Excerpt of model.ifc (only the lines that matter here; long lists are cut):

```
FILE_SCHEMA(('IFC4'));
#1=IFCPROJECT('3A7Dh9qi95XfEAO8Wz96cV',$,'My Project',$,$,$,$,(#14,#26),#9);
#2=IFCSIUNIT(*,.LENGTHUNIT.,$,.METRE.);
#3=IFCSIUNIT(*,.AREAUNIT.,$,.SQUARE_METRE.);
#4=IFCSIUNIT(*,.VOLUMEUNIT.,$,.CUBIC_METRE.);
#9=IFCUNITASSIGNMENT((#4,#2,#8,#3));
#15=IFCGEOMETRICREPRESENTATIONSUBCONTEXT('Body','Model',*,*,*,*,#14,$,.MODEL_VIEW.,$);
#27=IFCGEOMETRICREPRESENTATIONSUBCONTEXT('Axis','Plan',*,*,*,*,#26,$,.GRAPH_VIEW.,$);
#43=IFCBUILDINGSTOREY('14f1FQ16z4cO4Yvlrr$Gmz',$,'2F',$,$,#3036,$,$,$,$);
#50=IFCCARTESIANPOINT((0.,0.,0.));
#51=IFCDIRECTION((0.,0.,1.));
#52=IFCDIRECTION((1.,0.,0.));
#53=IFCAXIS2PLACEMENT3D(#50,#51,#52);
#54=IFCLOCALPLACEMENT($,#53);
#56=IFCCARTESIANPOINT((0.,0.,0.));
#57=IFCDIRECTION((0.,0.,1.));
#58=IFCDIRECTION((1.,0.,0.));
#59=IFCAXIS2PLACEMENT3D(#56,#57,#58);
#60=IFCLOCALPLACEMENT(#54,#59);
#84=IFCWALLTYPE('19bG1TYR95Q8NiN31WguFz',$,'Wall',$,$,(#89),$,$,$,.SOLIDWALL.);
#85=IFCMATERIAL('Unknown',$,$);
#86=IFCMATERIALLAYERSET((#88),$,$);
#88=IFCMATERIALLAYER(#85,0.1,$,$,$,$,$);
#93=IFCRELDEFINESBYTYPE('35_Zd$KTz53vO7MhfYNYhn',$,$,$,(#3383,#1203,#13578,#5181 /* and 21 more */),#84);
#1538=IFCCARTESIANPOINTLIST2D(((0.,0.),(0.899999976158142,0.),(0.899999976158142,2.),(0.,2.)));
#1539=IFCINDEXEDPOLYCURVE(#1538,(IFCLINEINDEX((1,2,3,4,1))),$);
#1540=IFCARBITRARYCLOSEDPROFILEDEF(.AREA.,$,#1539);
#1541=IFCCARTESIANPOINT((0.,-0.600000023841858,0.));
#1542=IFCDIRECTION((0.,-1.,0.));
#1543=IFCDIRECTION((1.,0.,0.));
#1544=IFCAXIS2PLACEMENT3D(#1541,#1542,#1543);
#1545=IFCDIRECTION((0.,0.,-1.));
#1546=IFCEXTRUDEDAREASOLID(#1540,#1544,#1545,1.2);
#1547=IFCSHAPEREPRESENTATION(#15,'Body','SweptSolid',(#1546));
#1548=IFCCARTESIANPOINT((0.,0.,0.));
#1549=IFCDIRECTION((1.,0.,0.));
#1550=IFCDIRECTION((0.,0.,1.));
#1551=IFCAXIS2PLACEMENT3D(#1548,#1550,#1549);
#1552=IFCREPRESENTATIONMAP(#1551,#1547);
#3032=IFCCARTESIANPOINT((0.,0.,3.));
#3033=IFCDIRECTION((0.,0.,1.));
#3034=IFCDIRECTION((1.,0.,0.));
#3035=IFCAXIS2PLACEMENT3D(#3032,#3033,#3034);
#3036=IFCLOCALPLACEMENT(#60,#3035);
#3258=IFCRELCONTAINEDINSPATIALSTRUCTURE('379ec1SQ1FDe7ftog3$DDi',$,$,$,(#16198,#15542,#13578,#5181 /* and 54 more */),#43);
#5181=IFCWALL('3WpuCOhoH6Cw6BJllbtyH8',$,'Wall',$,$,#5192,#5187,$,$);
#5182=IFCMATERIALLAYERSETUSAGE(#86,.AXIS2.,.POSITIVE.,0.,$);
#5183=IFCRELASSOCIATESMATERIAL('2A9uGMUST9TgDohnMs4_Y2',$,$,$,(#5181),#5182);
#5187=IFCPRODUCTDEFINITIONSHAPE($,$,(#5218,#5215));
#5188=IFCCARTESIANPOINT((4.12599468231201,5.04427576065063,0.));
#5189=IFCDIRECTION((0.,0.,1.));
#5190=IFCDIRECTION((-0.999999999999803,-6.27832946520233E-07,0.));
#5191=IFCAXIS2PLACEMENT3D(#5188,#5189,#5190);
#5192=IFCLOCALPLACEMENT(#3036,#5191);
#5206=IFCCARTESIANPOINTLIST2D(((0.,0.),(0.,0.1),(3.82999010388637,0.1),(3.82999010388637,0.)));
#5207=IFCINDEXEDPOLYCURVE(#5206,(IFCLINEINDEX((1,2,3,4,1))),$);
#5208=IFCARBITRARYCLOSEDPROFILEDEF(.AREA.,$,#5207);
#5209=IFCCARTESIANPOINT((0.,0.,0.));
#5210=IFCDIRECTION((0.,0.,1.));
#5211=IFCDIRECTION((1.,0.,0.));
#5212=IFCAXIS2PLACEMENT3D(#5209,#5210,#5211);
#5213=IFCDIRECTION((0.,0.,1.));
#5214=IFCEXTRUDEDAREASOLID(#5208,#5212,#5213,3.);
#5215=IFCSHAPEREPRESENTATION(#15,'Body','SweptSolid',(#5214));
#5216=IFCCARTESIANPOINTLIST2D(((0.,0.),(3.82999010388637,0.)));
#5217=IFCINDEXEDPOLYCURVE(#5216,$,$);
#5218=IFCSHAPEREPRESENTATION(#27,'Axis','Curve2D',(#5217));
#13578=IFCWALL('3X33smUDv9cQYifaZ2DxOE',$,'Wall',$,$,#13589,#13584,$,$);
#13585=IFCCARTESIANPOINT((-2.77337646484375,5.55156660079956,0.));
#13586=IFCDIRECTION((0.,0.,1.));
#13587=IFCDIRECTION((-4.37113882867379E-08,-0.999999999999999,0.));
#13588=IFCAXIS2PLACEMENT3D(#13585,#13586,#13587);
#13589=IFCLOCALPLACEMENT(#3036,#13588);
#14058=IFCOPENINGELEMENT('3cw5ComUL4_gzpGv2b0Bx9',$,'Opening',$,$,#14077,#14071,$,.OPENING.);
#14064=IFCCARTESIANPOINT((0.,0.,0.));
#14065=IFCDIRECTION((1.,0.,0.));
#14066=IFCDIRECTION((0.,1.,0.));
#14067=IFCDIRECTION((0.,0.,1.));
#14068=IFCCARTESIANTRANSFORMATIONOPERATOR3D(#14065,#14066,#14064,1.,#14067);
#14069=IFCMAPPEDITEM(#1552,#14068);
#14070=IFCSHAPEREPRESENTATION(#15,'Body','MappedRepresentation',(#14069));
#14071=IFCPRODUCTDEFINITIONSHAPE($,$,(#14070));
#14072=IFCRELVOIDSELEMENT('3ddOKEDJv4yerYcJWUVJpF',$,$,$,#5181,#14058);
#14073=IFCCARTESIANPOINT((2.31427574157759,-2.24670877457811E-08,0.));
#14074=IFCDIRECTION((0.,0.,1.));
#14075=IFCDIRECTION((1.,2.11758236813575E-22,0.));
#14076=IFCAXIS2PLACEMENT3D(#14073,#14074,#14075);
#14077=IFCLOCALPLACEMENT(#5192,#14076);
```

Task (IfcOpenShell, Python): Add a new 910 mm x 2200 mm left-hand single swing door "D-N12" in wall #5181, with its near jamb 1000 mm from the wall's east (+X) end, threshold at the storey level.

```python
import numpy as np
import ifcopenshell
import ifcopenshell.api.feature
import ifcopenshell.api.geometry
import ifcopenshell.api.root
import ifcopenshell.api.spatial
import ifcopenshell.geom
import ifcopenshell.util.element
import ifcopenshell.util.placement
import ifcopenshell.util.representation
import ifcopenshell.util.shape
import ifcopenshell.util.unit

model = ifcopenshell.open("model.ifc")
unit_scale = ifcopenshell.util.unit.calculate_unit_scale(model)
settings = ifcopenshell.geom.settings()


def volume(element):
    """Net volume in cubic metres, openings subtracted."""
    shape = ifcopenshell.geom.create_shape(settings, element)
    return ifcopenshell.util.shape.get_volume(shape.geometry)


wall = model.by_guid("3WpuCOhoH6Cw6BJllbtyH8")
storey = ifcopenshell.util.element.get_container(wall, ifc_class="IfcBuildingStorey")
context = ifcopenshell.util.representation.get_context(model, "Model", "Body", "MODEL_VIEW")
before = volume(wall)

width, height, from_end, sill = 0.91, 2.2, 1, 0.0  # metres

# The wall runs along its own X axis, and the end named is its -X end.
wall_shape = ifcopenshell.geom.create_shape(settings, wall)
x, y, z = ifcopenshell.util.shape.get_vertices(wall_shape.geometry).T
start = x.min() + from_end
face, thickness = float(y.min()), float(y.max() - y.min())
wall_matrix = ifcopenshell.util.placement.get_local_placement(wall.ObjectPlacement)
level = ifcopenshell.util.placement.get_local_placement(storey.ObjectPlacement)[2, 3]


def in_wall(x, y):
    """Placement at x, y metres in the wall's axes, at sill height."""
    matrix = wall_matrix.copy()
    matrix[:, 3] = wall_matrix @ np.array([x / unit_scale, y / unit_scale, 0.0, 1.0])
    matrix[2, 3] = level + sill / unit_scale
    return matrix


# Opening: a box that overshoots both wall faces by 50 mm.
opening = ifcopenshell.api.root.create_entity(model, ifc_class="IfcOpeningElement", predefined_type="OPENING")
box = ifcopenshell.api.geometry.add_wall_representation(
    model, context=context, length=width, height=height, thickness=thickness + 0.1
)
ifcopenshell.api.geometry.assign_representation(model, product=opening, representation=box)
ifcopenshell.api.geometry.edit_object_placement(model, product=opening, matrix=in_wall(start, face - 0.05), is_si=False)
ifcopenshell.api.feature.add_feature(model, feature=opening, element=wall)

door = ifcopenshell.api.root.create_entity(model, ifc_class="IfcDoor", name="D-N12", predefined_type="DOOR")
door.OverallWidth, door.OverallHeight = width / unit_scale, height / unit_scale
door.OperationType = "SINGLE_SWING_LEFT"
body = ifcopenshell.api.geometry.add_door_representation(
    model,
    context=context,
    overall_width=door.OverallWidth,
    overall_height=door.OverallHeight,
    operation_type="SINGLE_SWING_LEFT",
    lining_properties={"LiningDepth": thickness / unit_scale, "ThresholdDepth": thickness / unit_scale},
)
ifcopenshell.api.geometry.assign_representation(model, product=door, representation=body)
ifcopenshell.api.spatial.assign_container(model, products=[door], relating_structure=storey)
ifcopenshell.api.feature.add_filling(model, opening=opening, element=door)

# The lining spans the wall, so the door starts at the wall face.
ifcopenshell.api.geometry.edit_object_placement(model, product=door, matrix=in_wall(start, face), is_si=False)

after = volume(wall)

print(f"wall volume {before:.3f} -> {after:.3f} m3")

model.write("model_edited.ifc")
```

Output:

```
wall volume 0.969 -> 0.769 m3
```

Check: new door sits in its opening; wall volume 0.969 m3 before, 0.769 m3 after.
